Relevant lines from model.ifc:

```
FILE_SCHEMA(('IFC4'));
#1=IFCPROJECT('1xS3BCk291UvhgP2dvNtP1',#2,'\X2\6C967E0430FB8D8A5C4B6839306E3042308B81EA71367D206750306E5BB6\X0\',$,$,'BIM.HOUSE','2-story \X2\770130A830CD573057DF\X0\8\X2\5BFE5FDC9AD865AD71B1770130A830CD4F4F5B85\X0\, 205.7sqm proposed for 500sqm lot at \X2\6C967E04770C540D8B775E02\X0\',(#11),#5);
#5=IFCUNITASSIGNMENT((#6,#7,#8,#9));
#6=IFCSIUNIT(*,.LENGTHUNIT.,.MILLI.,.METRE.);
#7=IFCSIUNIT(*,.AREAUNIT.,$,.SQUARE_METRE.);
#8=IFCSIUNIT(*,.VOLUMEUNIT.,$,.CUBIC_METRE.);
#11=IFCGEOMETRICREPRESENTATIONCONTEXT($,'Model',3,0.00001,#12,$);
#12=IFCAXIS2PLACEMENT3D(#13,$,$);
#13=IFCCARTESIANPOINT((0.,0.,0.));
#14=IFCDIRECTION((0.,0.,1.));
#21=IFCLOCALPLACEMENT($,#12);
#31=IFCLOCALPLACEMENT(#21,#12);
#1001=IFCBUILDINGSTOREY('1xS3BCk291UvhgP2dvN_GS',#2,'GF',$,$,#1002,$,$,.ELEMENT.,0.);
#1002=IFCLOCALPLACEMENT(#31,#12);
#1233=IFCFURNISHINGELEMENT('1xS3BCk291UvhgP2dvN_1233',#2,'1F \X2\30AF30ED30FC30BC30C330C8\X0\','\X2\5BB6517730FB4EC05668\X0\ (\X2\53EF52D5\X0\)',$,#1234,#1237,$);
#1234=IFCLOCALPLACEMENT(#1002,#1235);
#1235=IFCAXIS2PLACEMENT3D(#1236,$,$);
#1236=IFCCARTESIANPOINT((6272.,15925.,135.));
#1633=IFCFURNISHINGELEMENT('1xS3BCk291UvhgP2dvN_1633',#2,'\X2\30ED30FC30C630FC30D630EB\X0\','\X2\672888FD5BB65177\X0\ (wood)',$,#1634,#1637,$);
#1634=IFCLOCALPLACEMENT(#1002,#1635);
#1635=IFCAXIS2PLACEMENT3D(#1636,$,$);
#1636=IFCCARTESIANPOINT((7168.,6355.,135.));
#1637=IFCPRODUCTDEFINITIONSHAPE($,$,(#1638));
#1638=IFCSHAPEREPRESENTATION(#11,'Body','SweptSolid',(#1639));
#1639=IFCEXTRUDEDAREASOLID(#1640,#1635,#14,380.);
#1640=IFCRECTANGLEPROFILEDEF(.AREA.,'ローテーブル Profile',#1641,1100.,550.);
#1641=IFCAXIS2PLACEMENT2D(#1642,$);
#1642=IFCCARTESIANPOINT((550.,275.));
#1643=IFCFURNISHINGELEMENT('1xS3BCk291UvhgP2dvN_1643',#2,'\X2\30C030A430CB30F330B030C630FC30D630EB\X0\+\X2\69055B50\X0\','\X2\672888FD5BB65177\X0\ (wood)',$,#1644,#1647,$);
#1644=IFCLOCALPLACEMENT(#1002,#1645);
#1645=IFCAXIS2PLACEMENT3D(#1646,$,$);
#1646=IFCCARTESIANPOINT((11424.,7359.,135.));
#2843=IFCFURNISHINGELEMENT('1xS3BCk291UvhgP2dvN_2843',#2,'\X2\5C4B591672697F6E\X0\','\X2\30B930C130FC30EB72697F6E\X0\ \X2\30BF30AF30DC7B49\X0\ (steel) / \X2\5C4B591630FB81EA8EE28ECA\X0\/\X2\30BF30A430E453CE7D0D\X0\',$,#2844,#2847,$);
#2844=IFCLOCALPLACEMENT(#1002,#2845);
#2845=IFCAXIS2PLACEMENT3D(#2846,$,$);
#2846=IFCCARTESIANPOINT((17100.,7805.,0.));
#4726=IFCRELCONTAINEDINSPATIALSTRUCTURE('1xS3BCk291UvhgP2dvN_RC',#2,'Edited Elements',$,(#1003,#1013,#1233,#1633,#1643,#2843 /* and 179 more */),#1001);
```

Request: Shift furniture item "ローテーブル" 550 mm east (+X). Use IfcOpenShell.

```python
import ifcopenshell
import ifcopenshell.api.geometry
import ifcopenshell.util.placement
import ifcopenshell.util.unit

model = ifcopenshell.open("model.ifc")
unit_scale = ifcopenshell.util.unit.calculate_unit_scale(model)

item = model.by_guid("1xS3BCk291UvhgP2dvN_1633")
matrix = ifcopenshell.util.placement.get_local_placement(item.ObjectPlacement)
matrix[0, 3] += 0.55 / unit_scale
ifcopenshell.api.geometry.edit_object_placement(model, product=item, matrix=matrix, is_si=False)

print(ifcopenshell.util.placement.get_local_placement(item.ObjectPlacement).round(3) + 0.0)

model.write("model_rev.ifc")
```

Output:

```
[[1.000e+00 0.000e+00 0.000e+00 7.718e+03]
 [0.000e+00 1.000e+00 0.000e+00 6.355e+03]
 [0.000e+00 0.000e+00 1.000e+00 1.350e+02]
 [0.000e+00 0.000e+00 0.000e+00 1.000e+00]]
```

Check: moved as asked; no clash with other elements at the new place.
